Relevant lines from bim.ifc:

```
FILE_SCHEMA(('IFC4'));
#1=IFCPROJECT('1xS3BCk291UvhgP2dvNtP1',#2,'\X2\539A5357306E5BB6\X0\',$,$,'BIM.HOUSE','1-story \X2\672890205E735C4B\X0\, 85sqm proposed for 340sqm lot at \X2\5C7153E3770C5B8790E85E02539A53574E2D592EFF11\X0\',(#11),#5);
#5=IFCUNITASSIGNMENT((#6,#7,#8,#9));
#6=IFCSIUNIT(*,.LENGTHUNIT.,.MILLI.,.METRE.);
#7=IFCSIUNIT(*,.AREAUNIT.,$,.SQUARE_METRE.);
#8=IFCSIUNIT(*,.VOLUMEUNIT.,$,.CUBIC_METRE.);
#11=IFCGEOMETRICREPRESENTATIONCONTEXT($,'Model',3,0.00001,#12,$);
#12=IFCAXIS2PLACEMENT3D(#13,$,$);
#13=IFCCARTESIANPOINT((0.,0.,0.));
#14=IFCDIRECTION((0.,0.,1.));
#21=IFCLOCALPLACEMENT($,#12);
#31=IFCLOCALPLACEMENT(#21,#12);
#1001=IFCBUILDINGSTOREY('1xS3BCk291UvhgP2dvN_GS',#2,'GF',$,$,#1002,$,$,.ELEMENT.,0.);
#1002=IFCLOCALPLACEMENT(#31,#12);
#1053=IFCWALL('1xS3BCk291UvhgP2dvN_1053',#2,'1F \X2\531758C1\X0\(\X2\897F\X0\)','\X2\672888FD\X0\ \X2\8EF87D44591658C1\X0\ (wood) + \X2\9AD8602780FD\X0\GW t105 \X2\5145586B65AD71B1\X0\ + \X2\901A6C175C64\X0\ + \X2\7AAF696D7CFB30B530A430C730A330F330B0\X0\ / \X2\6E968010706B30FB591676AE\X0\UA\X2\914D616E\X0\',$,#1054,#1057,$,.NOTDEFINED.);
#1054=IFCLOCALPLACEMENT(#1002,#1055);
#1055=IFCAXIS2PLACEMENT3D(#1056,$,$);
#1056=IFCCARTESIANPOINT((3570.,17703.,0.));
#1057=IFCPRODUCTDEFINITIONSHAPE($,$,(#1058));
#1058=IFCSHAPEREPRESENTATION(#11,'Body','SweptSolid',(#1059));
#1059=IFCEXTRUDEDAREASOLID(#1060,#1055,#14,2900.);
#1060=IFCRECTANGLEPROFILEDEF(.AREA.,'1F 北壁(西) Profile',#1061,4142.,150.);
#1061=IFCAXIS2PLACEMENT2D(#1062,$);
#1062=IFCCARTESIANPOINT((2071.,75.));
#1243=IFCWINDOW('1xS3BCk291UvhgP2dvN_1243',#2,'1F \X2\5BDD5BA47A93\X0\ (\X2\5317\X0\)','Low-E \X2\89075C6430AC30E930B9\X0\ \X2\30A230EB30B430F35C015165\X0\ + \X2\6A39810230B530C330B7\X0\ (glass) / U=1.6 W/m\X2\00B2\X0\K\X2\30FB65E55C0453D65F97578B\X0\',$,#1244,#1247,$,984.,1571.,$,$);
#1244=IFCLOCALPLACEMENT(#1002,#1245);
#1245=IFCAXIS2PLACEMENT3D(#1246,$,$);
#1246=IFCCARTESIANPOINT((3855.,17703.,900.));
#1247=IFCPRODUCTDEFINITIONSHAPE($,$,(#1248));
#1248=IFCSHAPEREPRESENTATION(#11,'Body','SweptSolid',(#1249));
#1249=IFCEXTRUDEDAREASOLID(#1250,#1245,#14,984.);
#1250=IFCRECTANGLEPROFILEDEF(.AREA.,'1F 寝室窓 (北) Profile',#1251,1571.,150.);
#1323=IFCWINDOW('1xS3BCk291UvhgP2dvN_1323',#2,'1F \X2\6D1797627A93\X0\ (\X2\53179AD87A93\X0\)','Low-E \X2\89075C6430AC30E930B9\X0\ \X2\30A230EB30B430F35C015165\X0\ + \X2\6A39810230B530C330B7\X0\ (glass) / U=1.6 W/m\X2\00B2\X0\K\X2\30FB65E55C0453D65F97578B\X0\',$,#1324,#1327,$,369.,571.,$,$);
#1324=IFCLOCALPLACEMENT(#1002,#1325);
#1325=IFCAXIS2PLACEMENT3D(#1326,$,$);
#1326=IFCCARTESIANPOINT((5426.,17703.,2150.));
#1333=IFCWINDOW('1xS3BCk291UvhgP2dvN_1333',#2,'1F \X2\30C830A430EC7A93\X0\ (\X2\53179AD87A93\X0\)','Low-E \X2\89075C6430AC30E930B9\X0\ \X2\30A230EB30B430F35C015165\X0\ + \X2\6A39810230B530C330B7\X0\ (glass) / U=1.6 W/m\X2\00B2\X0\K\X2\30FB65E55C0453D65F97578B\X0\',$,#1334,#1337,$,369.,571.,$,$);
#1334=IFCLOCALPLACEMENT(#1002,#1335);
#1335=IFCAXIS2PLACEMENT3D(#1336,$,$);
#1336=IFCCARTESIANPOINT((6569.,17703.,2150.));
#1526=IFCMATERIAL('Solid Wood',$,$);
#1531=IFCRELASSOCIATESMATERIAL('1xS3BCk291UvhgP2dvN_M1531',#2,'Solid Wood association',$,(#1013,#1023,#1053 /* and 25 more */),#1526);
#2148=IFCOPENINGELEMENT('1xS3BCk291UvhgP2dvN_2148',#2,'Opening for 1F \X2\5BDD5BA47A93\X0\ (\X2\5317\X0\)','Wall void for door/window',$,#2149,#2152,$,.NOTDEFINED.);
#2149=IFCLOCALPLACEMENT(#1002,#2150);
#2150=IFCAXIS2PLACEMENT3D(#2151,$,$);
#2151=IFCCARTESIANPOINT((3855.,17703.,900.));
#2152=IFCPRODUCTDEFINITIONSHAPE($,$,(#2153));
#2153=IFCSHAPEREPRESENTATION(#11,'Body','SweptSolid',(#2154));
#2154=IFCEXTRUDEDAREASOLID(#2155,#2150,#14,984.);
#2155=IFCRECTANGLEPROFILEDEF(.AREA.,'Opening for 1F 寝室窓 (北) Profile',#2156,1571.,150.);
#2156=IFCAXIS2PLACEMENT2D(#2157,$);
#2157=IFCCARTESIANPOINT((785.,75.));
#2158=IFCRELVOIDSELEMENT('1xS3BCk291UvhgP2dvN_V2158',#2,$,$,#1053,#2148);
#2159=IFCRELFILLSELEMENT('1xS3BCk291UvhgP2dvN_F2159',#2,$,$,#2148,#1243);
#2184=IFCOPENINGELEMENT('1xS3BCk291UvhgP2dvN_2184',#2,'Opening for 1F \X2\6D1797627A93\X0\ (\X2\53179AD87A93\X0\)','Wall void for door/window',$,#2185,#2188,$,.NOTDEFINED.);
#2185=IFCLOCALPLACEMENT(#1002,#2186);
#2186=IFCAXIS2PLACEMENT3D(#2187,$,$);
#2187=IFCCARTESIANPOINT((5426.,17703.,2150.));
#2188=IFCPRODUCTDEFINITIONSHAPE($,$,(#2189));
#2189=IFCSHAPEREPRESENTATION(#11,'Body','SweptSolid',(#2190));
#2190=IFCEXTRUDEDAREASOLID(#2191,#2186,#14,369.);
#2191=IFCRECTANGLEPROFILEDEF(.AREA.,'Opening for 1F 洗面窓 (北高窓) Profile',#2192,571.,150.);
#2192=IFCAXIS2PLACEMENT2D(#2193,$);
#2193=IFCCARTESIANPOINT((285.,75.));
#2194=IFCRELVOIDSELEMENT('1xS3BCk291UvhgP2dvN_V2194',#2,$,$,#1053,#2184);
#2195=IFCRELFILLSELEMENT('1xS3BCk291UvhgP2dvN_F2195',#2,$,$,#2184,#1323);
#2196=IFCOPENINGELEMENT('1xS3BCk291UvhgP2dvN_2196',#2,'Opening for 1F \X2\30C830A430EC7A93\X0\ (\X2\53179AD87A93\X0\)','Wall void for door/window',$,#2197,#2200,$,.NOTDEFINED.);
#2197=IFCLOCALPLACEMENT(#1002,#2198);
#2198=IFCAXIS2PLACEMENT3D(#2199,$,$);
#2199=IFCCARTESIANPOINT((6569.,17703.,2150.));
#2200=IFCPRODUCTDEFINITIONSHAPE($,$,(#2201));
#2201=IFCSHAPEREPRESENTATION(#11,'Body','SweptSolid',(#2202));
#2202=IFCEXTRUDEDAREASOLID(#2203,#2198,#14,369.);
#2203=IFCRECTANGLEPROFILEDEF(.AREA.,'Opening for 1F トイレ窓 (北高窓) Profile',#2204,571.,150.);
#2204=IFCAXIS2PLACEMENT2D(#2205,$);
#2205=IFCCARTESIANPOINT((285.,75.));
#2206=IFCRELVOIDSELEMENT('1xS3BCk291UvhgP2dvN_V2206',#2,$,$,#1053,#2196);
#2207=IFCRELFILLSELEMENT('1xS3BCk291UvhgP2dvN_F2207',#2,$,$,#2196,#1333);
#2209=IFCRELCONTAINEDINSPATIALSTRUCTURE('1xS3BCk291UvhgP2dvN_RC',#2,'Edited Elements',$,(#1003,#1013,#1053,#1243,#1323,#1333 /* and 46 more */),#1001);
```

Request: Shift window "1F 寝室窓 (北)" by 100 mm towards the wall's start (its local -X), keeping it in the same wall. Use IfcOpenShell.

```python
import ifcopenshell
import ifcopenshell.api.geometry
import ifcopenshell.util.placement
import ifcopenshell.util.unit

model = ifcopenshell.open("bim.ifc")
unit_scale = ifcopenshell.util.unit.calculate_unit_scale(model)

window = model.by_guid("1xS3BCk291UvhgP2dvN_1243")
opening = window.FillsVoids[0].RelatingOpeningElement
wall = opening.VoidsElements[0].RelatingBuildingElement

wall_matrix = ifcopenshell.util.placement.get_local_placement(wall.ObjectPlacement)
shift = wall_matrix[:3, 0] * -0.1 / unit_scale
before = ifcopenshell.util.placement.get_local_placement(window.ObjectPlacement)[:3, 3].copy()

# The window is not placed relative to its opening, so move both.
for product in (opening, window):
    matrix = ifcopenshell.util.placement.get_local_placement(product.ObjectPlacement)
    matrix[:3, 3] += shift
    ifcopenshell.api.geometry.edit_object_placement(model, product=product, matrix=matrix, is_si=False)

after = ifcopenshell.util.placement.get_local_placement(window.ObjectPlacement)[:3, 3]
print("window moved by", (after - before).round(3) + 0.0)

model.write("bim-out.ifc")
```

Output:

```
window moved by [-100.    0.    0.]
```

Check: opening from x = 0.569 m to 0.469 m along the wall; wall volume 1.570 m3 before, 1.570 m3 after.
